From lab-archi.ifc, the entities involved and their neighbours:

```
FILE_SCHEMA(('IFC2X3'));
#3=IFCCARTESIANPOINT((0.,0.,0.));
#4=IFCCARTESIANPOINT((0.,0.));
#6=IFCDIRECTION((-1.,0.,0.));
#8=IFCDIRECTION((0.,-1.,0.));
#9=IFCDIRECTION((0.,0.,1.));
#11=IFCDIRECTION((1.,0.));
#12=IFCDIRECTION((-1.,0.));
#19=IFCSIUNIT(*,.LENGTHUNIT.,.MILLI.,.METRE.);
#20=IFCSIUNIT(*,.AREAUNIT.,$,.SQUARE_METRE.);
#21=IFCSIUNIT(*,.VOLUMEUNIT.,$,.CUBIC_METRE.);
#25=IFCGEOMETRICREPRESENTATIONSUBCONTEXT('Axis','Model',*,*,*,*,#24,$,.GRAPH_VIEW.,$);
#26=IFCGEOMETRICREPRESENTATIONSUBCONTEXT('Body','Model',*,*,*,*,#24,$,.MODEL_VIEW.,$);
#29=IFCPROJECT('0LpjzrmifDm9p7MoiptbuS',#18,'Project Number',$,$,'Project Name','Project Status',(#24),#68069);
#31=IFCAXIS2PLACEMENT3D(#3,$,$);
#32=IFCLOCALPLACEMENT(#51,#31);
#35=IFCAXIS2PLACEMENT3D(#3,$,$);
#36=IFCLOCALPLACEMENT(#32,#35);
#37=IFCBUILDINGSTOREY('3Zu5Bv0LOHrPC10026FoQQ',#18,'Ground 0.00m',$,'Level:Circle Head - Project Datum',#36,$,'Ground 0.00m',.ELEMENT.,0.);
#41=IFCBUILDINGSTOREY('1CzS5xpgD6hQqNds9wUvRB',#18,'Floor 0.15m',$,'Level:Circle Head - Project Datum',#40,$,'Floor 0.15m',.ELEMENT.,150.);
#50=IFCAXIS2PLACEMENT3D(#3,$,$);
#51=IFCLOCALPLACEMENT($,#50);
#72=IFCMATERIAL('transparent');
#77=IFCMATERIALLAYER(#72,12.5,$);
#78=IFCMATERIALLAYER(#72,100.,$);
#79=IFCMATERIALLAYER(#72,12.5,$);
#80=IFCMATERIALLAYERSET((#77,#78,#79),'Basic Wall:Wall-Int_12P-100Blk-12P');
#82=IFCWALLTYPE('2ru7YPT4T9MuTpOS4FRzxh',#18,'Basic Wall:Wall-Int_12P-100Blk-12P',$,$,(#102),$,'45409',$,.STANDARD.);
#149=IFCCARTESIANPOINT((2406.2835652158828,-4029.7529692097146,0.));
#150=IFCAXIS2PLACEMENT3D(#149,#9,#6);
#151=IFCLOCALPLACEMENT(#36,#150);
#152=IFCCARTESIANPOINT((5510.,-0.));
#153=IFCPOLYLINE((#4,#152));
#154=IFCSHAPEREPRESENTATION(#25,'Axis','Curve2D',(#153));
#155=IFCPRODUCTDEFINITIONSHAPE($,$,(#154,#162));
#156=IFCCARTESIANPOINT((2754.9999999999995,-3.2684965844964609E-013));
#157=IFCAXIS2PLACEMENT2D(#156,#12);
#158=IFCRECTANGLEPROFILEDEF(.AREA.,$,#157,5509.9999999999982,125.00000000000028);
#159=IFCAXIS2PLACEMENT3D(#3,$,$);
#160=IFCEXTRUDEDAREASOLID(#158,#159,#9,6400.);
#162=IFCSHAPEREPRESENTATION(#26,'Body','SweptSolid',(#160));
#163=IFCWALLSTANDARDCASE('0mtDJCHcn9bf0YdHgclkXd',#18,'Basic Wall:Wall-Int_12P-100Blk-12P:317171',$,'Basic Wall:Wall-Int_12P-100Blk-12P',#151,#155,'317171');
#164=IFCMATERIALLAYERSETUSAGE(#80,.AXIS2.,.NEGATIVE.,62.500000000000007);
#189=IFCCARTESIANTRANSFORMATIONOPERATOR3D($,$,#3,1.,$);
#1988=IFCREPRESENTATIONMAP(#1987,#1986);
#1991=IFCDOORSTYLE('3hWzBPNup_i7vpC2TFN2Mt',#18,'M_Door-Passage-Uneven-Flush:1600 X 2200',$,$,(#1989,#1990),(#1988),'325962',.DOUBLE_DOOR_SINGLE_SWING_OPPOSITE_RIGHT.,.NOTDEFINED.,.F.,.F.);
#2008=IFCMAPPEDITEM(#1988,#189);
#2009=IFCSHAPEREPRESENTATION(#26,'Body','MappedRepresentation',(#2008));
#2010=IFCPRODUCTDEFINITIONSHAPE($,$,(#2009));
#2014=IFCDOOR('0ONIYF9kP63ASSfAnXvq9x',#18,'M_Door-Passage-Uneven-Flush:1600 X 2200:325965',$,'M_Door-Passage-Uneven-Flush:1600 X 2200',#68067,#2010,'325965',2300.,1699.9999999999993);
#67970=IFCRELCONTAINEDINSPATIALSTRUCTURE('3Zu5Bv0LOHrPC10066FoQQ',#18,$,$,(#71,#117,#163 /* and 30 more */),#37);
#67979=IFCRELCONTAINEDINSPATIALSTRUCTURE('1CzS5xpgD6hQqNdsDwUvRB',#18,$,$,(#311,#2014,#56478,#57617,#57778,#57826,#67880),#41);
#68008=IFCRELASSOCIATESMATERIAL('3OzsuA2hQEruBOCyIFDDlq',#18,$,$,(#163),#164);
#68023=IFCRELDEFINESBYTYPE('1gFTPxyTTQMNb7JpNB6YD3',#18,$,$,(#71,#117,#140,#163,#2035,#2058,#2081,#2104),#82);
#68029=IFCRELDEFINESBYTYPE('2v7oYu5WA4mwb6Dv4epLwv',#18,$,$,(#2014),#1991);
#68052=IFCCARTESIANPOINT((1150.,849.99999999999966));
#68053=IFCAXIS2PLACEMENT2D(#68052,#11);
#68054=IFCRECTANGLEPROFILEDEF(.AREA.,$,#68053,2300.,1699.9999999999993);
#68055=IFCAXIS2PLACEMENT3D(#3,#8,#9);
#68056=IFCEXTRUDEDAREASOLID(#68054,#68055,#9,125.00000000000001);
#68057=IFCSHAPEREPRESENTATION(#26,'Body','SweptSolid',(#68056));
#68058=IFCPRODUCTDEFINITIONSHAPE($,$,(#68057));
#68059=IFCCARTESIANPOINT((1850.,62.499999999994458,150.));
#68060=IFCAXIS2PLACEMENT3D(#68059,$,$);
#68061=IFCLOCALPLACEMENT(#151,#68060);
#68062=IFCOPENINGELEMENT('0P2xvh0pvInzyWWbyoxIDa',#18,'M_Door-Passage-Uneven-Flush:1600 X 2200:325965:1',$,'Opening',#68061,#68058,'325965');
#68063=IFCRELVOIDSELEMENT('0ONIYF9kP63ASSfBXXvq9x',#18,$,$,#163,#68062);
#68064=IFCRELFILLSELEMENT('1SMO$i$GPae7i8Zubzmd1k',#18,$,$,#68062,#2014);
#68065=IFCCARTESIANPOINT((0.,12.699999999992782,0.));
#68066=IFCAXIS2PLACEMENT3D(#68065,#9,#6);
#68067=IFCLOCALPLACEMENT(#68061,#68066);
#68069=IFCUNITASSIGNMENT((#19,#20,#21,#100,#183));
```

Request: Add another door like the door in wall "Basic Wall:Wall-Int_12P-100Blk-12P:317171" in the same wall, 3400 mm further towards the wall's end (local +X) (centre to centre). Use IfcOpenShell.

```python
import ifcopenshell
import ifcopenshell.api.feature
import ifcopenshell.api.geometry
import ifcopenshell.api.root
import ifcopenshell.geom
import ifcopenshell.util.element
import ifcopenshell.util.placement
import ifcopenshell.util.shape
import ifcopenshell.util.unit

model = ifcopenshell.open("lab-archi.ifc")
unit_scale = ifcopenshell.util.unit.calculate_unit_scale(model)
settings = ifcopenshell.geom.settings()


def volume(element):
    """Net volume in cubic metres, openings subtracted."""
    shape = ifcopenshell.geom.create_shape(settings, element)
    return ifcopenshell.util.shape.get_volume(shape.geometry)


def reuse_history(source, copy):
    """copy_class also copies each property set's owner history, people and application; keep the originals."""
    for rel in copy.IsDefinedBy:
        if rel.is_a("IfcRelDefinesByProperties") and (history := rel.RelatingPropertyDefinition.OwnerHistory):
            rel.RelatingPropertyDefinition.OwnerHistory = source.OwnerHistory
            ifcopenshell.util.element.remove_deep2(model, history)


door = model.by_id(2014)
opening = door.FillsVoids[0].RelatingOpeningElement
wall = opening.VoidsElements[0].RelatingBuildingElement
before = volume(wall)
shift = ifcopenshell.util.placement.get_local_placement(wall.ObjectPlacement)[:3, 0] * 3.4 / unit_scale

# copy_class copies the void relationship, type, container and properties, but no geometry.
new_opening = ifcopenshell.api.root.copy_class(model, product=opening)
new_opening.Representation = ifcopenshell.util.element.copy_deep(
    model, opening.Representation, exclude=["IfcGeometricRepresentationContext", "IfcRepresentationMap"]
)
new_opening.Name = "M_Door-Passage-Uneven-Flush:1600 X 2200"
new_opening.Tag = None
new_door = ifcopenshell.api.root.copy_class(model, product=door)
new_door.Representation = ifcopenshell.util.element.copy_deep(
    model, door.Representation, exclude=["IfcGeometricRepresentationContext", "IfcRepresentationMap"]
)
new_door.Name = "M_Door-Passage-Uneven-Flush:1600 X 2200"
new_door.Tag = None
reuse_history(door, new_door)
fills = ifcopenshell.api.feature.add_filling(model, opening=new_opening, element=new_door)
fills.OwnerHistory = new_door.OwnerHistory  # required in IFC2X3

for old, new in ((opening, new_opening), (door, new_door)):
    matrix = ifcopenshell.util.placement.get_local_placement(old.ObjectPlacement)
    matrix[:3, 3] += shift
    ifcopenshell.api.geometry.edit_object_placement(model, product=new, matrix=matrix, is_si=False)

after = volume(wall)

print(f"wall volume {before:.3f} -> {after:.3f} m3")

model.write("lab-archi-out.ifc")
```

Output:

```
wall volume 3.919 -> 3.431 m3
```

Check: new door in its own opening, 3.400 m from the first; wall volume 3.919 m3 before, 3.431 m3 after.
